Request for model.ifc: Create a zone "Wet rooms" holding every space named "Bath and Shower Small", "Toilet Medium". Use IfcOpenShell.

First a look at what the model holds.

```python
import ifcopenshell

model = ifcopenshell.open("model.ifc")
print(model.schema)
seen = {}
for space in model.by_type("IfcSpace"):
    seen[space.LongName] = seen.get(space.LongName, 0) + 1
for name, count in sorted(seen.items(), key=str):
    print(count, "x", name)
print("zones:", [z.Name for z in model.by_type("IfcZone")][:20])
```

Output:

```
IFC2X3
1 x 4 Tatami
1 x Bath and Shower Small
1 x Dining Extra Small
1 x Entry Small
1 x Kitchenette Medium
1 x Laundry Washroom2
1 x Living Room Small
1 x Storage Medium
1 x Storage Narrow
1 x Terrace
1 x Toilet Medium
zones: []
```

```python
import ifcopenshell
import ifcopenshell.api.group
import ifcopenshell.api.root

model = ifcopenshell.open("model.ifc")

names = {"Bath and Shower Small", "Toilet Medium"}
spaces = [s for s in model.by_type("IfcSpace") if s.LongName in names]

zone = ifcopenshell.api.root.create_entity(model, ifc_class="IfcZone", name="Wet rooms")
ifcopenshell.api.group.assign_group(model, products=spaces, group=zone)
print(len(spaces), "spaces in", zone.Name)

model.write("model_edited.ifc")
```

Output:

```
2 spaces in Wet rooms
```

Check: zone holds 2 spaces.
